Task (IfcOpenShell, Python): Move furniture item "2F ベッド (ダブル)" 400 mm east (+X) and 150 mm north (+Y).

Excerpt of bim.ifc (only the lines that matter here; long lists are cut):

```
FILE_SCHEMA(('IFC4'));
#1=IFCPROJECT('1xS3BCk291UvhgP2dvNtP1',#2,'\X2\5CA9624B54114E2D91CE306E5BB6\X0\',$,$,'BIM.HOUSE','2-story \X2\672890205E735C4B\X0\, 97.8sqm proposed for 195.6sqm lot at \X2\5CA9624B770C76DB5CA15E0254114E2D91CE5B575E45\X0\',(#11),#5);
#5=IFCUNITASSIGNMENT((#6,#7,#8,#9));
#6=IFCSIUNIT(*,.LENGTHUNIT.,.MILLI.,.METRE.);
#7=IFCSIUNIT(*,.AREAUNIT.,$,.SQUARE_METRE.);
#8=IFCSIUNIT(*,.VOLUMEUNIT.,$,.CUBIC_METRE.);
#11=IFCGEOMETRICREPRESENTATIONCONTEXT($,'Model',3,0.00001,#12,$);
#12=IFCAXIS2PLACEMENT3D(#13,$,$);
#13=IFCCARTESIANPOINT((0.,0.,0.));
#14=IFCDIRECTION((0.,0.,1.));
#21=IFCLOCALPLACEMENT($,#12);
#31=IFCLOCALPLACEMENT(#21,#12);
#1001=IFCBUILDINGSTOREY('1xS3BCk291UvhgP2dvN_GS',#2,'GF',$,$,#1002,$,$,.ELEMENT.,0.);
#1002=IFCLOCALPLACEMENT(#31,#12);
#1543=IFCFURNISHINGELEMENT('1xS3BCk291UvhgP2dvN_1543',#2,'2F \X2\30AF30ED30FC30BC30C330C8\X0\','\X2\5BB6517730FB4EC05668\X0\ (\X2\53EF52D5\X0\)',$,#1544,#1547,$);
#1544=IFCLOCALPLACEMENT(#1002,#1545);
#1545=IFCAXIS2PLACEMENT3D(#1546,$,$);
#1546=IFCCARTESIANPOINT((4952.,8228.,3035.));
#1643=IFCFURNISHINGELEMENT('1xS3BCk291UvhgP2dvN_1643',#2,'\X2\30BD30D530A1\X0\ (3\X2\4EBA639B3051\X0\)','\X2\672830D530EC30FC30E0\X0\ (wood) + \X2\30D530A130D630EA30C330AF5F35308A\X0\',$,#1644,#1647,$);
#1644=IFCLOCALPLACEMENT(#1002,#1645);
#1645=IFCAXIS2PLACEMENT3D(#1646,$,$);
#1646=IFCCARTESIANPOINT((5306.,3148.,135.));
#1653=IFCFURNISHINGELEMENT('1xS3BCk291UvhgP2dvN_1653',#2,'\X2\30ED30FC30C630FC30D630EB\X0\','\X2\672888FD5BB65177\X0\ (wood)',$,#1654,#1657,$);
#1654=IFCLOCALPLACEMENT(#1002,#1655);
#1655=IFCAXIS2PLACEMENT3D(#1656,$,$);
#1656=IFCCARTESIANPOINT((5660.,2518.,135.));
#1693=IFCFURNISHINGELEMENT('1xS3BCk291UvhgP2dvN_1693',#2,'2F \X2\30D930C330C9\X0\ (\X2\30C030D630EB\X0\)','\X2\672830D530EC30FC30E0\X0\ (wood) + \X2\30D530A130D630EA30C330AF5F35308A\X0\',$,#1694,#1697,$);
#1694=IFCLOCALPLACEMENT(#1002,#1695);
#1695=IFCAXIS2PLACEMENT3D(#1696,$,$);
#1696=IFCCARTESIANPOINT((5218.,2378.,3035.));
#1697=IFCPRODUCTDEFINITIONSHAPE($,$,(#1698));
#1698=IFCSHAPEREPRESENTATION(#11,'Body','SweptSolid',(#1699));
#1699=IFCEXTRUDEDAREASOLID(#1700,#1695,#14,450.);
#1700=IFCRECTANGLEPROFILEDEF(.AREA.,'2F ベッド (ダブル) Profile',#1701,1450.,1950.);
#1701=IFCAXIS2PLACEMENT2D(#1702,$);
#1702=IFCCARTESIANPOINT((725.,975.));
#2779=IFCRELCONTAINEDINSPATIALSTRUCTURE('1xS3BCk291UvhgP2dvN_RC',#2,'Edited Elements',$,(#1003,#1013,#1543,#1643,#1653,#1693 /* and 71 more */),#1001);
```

```python
import ifcopenshell
import ifcopenshell.api.geometry
import ifcopenshell.util.placement
import ifcopenshell.util.unit

model = ifcopenshell.open("bim.ifc")
unit_scale = ifcopenshell.util.unit.calculate_unit_scale(model)

item = model.by_id(1693)
matrix = ifcopenshell.util.placement.get_local_placement(item.ObjectPlacement)
matrix[0, 3] += 0.4 / unit_scale
matrix[1, 3] += 0.15 / unit_scale
ifcopenshell.api.geometry.edit_object_placement(model, product=item, matrix=matrix, is_si=False)

print(ifcopenshell.util.placement.get_local_placement(item.ObjectPlacement).round(3) + 0.0)

model.write("bim_rev.ifc")
```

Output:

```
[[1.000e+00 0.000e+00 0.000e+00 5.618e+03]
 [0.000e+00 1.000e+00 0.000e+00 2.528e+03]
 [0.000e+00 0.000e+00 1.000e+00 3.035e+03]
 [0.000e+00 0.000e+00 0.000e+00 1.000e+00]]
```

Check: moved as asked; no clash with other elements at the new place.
